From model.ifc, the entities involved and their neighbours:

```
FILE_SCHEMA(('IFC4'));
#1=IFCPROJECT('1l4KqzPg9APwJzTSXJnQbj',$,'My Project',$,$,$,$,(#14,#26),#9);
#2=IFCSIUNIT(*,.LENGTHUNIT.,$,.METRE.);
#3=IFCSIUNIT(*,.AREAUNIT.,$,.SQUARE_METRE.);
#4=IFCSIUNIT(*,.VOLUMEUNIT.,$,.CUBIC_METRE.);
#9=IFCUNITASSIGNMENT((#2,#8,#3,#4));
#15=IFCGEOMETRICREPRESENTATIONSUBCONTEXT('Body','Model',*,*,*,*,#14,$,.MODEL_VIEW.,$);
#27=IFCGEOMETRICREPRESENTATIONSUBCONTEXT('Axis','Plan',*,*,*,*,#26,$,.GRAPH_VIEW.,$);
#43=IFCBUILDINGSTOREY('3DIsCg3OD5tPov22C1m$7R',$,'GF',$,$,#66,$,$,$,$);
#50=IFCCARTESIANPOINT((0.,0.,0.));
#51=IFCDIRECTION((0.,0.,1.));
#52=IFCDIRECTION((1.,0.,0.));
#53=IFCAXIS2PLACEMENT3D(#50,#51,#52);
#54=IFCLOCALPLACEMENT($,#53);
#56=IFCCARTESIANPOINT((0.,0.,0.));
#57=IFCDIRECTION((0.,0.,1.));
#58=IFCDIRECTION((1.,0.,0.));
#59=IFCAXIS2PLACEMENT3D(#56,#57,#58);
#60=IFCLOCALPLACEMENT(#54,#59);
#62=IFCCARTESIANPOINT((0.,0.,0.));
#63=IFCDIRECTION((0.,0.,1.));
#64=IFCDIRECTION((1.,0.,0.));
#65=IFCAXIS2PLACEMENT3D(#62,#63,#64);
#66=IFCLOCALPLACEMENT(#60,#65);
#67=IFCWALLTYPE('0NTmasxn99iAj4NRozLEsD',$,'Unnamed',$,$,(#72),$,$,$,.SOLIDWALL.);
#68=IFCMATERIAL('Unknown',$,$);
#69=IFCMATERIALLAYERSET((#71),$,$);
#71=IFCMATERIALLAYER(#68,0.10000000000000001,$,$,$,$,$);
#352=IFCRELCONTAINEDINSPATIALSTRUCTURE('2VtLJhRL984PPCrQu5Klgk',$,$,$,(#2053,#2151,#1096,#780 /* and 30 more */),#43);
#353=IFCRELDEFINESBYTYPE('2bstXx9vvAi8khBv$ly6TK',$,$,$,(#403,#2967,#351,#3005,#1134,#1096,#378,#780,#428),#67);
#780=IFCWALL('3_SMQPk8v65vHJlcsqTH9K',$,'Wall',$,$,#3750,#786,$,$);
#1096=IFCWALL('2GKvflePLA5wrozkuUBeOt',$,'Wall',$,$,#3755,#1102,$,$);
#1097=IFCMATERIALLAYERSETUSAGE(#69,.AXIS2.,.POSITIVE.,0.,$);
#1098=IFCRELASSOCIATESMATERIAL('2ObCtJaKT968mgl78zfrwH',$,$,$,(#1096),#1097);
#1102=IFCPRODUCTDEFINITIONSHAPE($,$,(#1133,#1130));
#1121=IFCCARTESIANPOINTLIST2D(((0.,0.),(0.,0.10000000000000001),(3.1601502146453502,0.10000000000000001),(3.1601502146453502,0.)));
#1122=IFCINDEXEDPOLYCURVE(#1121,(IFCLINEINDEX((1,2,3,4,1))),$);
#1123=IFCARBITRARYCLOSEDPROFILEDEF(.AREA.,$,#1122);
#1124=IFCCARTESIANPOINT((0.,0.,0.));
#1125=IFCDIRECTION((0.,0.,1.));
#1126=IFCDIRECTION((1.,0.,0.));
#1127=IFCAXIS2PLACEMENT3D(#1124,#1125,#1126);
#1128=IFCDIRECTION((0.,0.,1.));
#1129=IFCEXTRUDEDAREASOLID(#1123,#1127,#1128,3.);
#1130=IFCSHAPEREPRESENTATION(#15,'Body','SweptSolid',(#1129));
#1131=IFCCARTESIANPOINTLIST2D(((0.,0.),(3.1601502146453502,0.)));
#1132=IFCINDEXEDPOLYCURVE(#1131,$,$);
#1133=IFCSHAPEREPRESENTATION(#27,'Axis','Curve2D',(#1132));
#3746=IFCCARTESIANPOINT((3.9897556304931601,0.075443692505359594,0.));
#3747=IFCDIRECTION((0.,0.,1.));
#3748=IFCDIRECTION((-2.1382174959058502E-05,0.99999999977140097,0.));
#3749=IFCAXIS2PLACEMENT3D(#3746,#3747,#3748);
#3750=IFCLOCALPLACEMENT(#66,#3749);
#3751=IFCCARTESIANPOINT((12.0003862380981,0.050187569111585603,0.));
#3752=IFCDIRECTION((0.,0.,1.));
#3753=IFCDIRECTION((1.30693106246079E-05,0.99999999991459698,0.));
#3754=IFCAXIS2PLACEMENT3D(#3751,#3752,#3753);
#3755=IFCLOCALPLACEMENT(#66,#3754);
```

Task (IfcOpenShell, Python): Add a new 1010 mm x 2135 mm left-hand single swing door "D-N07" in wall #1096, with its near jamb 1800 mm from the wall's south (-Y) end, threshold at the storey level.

```python
import numpy as np
import ifcopenshell
import ifcopenshell.api.feature
import ifcopenshell.api.geometry
import ifcopenshell.api.root
import ifcopenshell.api.spatial
import ifcopenshell.geom
import ifcopenshell.util.element
import ifcopenshell.util.placement
import ifcopenshell.util.representation
import ifcopenshell.util.shape
import ifcopenshell.util.unit

model = ifcopenshell.open("model.ifc")
unit_scale = ifcopenshell.util.unit.calculate_unit_scale(model)
settings = ifcopenshell.geom.settings()


def volume(element):
    """Net volume in cubic metres, openings subtracted."""
    shape = ifcopenshell.geom.create_shape(settings, element)
    return ifcopenshell.util.shape.get_volume(shape.geometry)


wall = model.by_guid("2GKvflePLA5wrozkuUBeOt")
storey = ifcopenshell.util.element.get_container(wall, ifc_class="IfcBuildingStorey")
context = ifcopenshell.util.representation.get_context(model, "Model", "Body", "MODEL_VIEW")
before = volume(wall)

width, height, from_end, sill = 1.01, 2.135, 1.8, 0.0  # metres

# The wall runs along its own X axis, and the end named is its -X end.
wall_shape = ifcopenshell.geom.create_shape(settings, wall)
x, y, z = ifcopenshell.util.shape.get_vertices(wall_shape.geometry).T
start = x.min() + from_end
face, thickness = float(y.min()), float(y.max() - y.min())
wall_matrix = ifcopenshell.util.placement.get_local_placement(wall.ObjectPlacement)
level = ifcopenshell.util.placement.get_local_placement(storey.ObjectPlacement)[2, 3]


def in_wall(x, y):
    """Placement at x, y metres in the wall's axes, at sill height."""
    matrix = wall_matrix.copy()
    matrix[:, 3] = wall_matrix @ np.array([x / unit_scale, y / unit_scale, 0.0, 1.0])
    matrix[2, 3] = level + sill / unit_scale
    return matrix


# Opening: a box that overshoots both wall faces by 50 mm.
opening = ifcopenshell.api.root.create_entity(model, ifc_class="IfcOpeningElement", predefined_type="OPENING")
box = ifcopenshell.api.geometry.add_wall_representation(
    model, context=context, length=width, height=height, thickness=thickness + 0.1
)
ifcopenshell.api.geometry.assign_representation(model, product=opening, representation=box)
ifcopenshell.api.geometry.edit_object_placement(model, product=opening, matrix=in_wall(start, face - 0.05), is_si=False)
ifcopenshell.api.feature.add_feature(model, feature=opening, element=wall)

door = ifcopenshell.api.root.create_entity(model, ifc_class="IfcDoor", name="D-N07", predefined_type="DOOR")
door.OverallWidth, door.OverallHeight = width / unit_scale, height / unit_scale
door.OperationType = "SINGLE_SWING_LEFT"
body = ifcopenshell.api.geometry.add_door_representation(
    model,
    context=context,
    overall_width=door.OverallWidth,
    overall_height=door.OverallHeight,
    operation_type="SINGLE_SWING_LEFT",
    lining_properties={"LiningDepth": thickness / unit_scale, "ThresholdDepth": thickness / unit_scale},
)
ifcopenshell.api.geometry.assign_representation(model, product=door, representation=body)
ifcopenshell.api.spatial.assign_container(model, products=[door], relating_structure=storey)
ifcopenshell.api.feature.add_filling(model, opening=opening, element=door)

# The lining spans the wall, so the door starts at the wall face.
ifcopenshell.api.geometry.edit_object_placement(model, product=door, matrix=in_wall(start, face), is_si=False)

after = volume(wall)

print(f"wall volume {before:.3f} -> {after:.3f} m3")

model.write("model_edited.ifc")
```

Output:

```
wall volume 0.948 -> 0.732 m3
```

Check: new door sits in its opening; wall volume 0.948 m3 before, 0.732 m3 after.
